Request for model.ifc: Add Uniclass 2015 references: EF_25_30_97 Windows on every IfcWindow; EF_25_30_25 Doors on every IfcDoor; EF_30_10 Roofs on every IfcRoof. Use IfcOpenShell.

First a look at what the model holds.

```python
import ifcopenshell

model = ifcopenshell.open("model.ifc")
print(model.schema)
print("classifications:", [c.Name for c in model.by_type("IfcClassification")])
for ifc_class in ("IfcDoor", "IfcRoof", "IfcStair", "IfcWall", "IfcWindow"):
    print(ifc_class, len(model.by_type(ifc_class)))
```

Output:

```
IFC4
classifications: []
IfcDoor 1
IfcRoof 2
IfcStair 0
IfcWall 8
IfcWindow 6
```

```python
import ifcopenshell
import ifcopenshell.api.classification

model = ifcopenshell.open("model.ifc")

system = ifcopenshell.api.classification.add_classification(model, classification="Uniclass 2015")

codes = {
    "IfcWindow": ("EF_25_30_97", "Windows"),
    "IfcDoor": ("EF_25_30_25", "Doors"),
    "IfcRoof": ("EF_30_10", "Roofs"),
}
for ifc_class, (code, name) in codes.items():
    products = model.by_type(ifc_class)
    ifcopenshell.api.classification.add_reference(
        model, products=products, classification=system, identification=code, name=name
    )
    print(code, len(products))

model.write("model_updated.ifc")
```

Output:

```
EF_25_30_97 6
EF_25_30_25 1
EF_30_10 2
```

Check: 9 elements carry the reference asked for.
